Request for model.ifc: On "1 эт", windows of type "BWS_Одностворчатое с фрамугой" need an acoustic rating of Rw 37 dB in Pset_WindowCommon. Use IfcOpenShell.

First a look at what the model holds.

```python
import ifcopenshell
import ifcopenshell.util.element

model = ifcopenshell.open("model.ifc")
print(model.schema)
storey = next(s for s in model.by_type("IfcBuildingStorey") if s.Name == "1 эт")
windows = [e for e in ifcopenshell.util.element.get_decomposition(storey) if e.is_a("IfcWindow")]
seen = {}
for e in windows:
    element_type = ifcopenshell.util.element.get_type(e)
    key = (element_type.Name if element_type != e and element_type else None, ifcopenshell.util.element.get_pset(e, "Pset_WindowCommon", "AcousticRating"))
    seen[key] = seen.get(key, 0) + 1
for (name, value), count in sorted(seen.items(), key=str):
    print(count, "x", name, "|", value)
```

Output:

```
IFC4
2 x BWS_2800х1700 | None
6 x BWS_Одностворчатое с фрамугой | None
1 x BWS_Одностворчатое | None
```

```python
import ifcopenshell
import ifcopenshell.api.pset
import ifcopenshell.util.element

model = ifcopenshell.open("model.ifc")

storey = next(s for s in model.by_type("IfcBuildingStorey") if s.Name == "1 эт")
windows = [e for e in ifcopenshell.util.element.get_decomposition(storey) if e.is_a("IfcWindow")]

count = 0
for e in windows:
    element_type = ifcopenshell.util.element.get_type(e)
    if element_type in (None, e) or element_type.Name != "BWS_Одностворчатое с фрамугой":
        continue
    # add_pset returns the element's existing set when there is one.
    pset = ifcopenshell.api.pset.add_pset(model, product=e, name="Pset_WindowCommon")
    ifcopenshell.api.pset.edit_pset(model, pset=pset, properties={"AcousticRating": "Rw 37 dB"})
    count += 1

print(count, "windows updated")

model.write("model_updated.ifc")
```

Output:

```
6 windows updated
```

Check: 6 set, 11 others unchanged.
